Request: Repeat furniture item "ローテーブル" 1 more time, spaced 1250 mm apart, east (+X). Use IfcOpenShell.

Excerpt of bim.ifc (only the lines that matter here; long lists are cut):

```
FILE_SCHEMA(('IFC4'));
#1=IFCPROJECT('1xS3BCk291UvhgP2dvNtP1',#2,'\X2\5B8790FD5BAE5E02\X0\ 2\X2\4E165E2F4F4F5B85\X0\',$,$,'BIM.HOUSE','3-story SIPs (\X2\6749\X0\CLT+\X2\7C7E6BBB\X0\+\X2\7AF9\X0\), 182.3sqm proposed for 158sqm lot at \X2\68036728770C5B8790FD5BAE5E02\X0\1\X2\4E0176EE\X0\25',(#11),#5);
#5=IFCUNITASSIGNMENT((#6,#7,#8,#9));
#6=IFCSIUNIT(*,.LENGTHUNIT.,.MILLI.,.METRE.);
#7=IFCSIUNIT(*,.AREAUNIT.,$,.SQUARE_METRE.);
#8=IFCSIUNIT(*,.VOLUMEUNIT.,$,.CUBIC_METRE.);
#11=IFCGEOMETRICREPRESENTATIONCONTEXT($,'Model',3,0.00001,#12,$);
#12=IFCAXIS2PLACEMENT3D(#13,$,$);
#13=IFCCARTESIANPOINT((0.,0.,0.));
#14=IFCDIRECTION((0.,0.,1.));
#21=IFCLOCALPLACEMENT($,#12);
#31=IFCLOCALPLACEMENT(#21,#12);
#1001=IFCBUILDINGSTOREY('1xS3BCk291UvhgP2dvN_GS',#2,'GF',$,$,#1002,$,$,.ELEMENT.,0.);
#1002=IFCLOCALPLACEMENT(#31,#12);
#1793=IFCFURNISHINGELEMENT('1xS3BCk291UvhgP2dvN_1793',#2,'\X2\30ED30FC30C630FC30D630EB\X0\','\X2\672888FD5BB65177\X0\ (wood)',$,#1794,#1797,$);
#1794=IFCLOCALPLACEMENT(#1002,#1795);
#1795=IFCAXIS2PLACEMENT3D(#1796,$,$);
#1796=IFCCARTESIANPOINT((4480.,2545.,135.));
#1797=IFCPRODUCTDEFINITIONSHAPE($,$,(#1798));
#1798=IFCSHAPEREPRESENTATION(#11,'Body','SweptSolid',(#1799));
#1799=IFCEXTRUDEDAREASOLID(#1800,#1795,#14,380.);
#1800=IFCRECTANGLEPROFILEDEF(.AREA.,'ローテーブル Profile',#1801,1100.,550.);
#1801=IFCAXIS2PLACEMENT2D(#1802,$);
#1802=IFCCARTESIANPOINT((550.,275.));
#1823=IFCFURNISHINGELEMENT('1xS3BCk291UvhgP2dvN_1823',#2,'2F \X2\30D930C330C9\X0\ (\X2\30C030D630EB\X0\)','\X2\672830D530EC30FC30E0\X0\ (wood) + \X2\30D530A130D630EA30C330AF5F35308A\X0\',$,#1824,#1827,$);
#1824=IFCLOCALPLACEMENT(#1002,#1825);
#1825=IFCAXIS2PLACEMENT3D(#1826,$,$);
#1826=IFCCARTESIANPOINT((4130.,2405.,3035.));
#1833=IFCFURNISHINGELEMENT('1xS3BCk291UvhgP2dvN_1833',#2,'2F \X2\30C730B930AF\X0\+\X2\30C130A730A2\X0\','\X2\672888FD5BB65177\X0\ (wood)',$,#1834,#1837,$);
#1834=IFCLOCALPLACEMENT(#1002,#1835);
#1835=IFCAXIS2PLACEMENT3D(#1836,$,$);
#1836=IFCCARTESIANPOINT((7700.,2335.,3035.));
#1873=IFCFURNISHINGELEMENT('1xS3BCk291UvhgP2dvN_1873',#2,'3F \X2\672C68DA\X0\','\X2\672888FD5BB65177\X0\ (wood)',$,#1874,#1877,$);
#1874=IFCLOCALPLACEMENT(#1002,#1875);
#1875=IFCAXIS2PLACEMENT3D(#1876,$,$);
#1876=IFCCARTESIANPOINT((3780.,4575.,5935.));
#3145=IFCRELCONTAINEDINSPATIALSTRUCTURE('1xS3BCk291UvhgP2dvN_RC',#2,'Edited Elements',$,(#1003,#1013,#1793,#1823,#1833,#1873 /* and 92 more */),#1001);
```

```python
import numpy as np
import ifcopenshell
import ifcopenshell.api.geometry
import ifcopenshell.api.root
import ifcopenshell.util.element
import ifcopenshell.util.placement

model = ifcopenshell.open("bim.ifc")


def reuse_history(source, copy):
    """copy_class also copies each property set's owner history, people and application; keep the originals."""
    for rel in copy.IsDefinedBy:
        if rel.is_a("IfcRelDefinesByProperties") and (history := rel.RelatingPropertyDefinition.OwnerHistory):
            rel.RelatingPropertyDefinition.OwnerHistory = source.OwnerHistory
            ifcopenshell.util.element.remove_deep2(model, history)


source = model.by_guid("1xS3BCk291UvhgP2dvN_1793")
base = ifcopenshell.util.placement.get_local_placement(source.ObjectPlacement)
step = np.array([1.0, 0.0, 0.0]) * 1250.0

for i in range(1, 2):
    copy = ifcopenshell.api.root.copy_class(model, product=source)
    copy.Representation = ifcopenshell.util.element.copy_deep(
        model, source.Representation, exclude=["IfcGeometricRepresentationContext", "IfcRepresentationMap"]
    )
    reuse_history(source, copy)
    matrix = base.copy()
    matrix[:3, 3] += i * step
    print("added at", matrix[:3, 3].round(3) + 0.0)
    ifcopenshell.api.geometry.edit_object_placement(model, product=copy, matrix=matrix, is_si=False)

model.write("bim_v2.ifc")
```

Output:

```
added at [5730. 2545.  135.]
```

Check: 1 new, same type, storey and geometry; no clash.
